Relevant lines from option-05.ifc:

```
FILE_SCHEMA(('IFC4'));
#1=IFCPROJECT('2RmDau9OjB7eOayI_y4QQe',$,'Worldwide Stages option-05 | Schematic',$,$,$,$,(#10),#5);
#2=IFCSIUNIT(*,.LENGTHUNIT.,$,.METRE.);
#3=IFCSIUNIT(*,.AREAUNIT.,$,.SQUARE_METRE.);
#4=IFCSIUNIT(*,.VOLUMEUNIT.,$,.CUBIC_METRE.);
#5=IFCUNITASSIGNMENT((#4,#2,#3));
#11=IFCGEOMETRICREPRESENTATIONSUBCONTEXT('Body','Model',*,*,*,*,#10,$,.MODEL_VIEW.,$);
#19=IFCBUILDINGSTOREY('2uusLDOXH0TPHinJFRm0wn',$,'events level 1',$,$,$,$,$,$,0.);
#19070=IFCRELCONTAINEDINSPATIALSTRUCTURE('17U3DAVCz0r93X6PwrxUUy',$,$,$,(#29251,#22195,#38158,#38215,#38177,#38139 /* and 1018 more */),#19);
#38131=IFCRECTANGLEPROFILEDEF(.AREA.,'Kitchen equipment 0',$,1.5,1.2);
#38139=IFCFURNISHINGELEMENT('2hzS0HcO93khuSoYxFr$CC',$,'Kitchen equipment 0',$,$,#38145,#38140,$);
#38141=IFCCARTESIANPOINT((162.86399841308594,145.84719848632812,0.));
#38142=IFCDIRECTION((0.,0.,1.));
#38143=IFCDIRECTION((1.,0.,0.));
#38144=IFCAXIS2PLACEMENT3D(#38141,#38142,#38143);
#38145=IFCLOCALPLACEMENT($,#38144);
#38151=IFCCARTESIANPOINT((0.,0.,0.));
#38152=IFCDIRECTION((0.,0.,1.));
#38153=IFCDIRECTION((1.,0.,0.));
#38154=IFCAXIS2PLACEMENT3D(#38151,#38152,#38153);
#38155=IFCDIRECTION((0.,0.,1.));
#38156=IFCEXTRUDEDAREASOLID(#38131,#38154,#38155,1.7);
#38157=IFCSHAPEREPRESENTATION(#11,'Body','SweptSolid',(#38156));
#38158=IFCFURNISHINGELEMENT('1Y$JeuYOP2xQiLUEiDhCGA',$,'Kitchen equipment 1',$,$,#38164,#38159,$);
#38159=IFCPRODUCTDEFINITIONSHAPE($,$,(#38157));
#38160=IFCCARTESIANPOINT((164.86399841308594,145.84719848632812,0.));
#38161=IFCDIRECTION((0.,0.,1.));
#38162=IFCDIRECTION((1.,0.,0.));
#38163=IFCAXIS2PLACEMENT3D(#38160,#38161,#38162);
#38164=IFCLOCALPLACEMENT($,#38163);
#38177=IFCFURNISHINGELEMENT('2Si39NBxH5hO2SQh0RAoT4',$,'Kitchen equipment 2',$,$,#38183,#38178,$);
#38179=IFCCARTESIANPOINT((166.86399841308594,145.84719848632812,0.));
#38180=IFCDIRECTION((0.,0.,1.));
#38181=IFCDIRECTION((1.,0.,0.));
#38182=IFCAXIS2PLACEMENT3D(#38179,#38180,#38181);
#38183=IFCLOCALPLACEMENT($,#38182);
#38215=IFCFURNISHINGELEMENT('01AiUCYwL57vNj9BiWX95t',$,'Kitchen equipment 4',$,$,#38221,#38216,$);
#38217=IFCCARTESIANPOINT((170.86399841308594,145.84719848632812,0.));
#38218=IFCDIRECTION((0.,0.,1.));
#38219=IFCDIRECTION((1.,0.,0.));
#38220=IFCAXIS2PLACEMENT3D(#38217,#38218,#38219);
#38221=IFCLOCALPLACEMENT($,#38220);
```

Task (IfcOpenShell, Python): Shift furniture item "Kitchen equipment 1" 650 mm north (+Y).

```python
import ifcopenshell
import ifcopenshell.api.geometry
import ifcopenshell.util.placement
import ifcopenshell.util.unit

model = ifcopenshell.open("option-05.ifc")
unit_scale = ifcopenshell.util.unit.calculate_unit_scale(model)

item = model.by_guid("1Y$JeuYOP2xQiLUEiDhCGA")
matrix = ifcopenshell.util.placement.get_local_placement(item.ObjectPlacement)
matrix[1, 3] += 0.65 / unit_scale
ifcopenshell.api.geometry.edit_object_placement(model, product=item, matrix=matrix, is_si=False)

print(ifcopenshell.util.placement.get_local_placement(item.ObjectPlacement).round(3) + 0.0)

model.write("option-05_edited.ifc")
```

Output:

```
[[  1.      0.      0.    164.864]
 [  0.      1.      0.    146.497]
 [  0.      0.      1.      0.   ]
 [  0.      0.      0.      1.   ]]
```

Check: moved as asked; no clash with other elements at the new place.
